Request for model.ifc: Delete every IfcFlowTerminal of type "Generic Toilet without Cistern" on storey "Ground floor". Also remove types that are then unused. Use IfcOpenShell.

First a look at what the model holds.

```python
import ifcopenshell
import ifcopenshell.util.element

model = ifcopenshell.open("model.ifc")
print(model.schema)
storey = next(s for s in model.by_type("IfcBuildingStorey") if s.Name == "Ground floor")
terminals = [e for e in ifcopenshell.util.element.get_decomposition(storey) if e.is_a("IfcFlowTerminal")]
seen = {}
for e in terminals:
    element_type = ifcopenshell.util.element.get_type(e)
    name = element_type.Name if element_type not in (None, e) else None
    seen[name] = seen.get(name, 0) + 1
for name, count in sorted(seen.items(), key=str):
    print(count, "x", name)
```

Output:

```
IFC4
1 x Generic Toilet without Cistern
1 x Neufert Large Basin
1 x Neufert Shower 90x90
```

```python
import ifcopenshell
import ifcopenshell.api.root
import ifcopenshell.util.element

model = ifcopenshell.open("model.ifc")

storey = next(s for s in model.by_type("IfcBuildingStorey") if s.Name == "Ground floor")
terminals = [e for e in ifcopenshell.util.element.get_decomposition(storey) if e.is_a("IfcFlowTerminal")]
targets = [e for e in terminals if (t := ifcopenshell.util.element.get_type(e)) not in (None, e) and t.Name == "Generic Toilet without Cistern"]
types = {ifcopenshell.util.element.get_type(e) for e in targets} - {None, *targets}

for e in targets:
    ifcopenshell.api.root.remove_product(model, product=e)
print(len(targets), "removed")

unused = [t for t in types if not ifcopenshell.util.element.get_types(t)]
for t in unused:
    ifcopenshell.api.root.remove_product(model, product=t)
print(len(unused), "unused types removed")

model.write("model_v2.ifc")
```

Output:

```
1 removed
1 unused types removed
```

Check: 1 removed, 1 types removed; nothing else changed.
